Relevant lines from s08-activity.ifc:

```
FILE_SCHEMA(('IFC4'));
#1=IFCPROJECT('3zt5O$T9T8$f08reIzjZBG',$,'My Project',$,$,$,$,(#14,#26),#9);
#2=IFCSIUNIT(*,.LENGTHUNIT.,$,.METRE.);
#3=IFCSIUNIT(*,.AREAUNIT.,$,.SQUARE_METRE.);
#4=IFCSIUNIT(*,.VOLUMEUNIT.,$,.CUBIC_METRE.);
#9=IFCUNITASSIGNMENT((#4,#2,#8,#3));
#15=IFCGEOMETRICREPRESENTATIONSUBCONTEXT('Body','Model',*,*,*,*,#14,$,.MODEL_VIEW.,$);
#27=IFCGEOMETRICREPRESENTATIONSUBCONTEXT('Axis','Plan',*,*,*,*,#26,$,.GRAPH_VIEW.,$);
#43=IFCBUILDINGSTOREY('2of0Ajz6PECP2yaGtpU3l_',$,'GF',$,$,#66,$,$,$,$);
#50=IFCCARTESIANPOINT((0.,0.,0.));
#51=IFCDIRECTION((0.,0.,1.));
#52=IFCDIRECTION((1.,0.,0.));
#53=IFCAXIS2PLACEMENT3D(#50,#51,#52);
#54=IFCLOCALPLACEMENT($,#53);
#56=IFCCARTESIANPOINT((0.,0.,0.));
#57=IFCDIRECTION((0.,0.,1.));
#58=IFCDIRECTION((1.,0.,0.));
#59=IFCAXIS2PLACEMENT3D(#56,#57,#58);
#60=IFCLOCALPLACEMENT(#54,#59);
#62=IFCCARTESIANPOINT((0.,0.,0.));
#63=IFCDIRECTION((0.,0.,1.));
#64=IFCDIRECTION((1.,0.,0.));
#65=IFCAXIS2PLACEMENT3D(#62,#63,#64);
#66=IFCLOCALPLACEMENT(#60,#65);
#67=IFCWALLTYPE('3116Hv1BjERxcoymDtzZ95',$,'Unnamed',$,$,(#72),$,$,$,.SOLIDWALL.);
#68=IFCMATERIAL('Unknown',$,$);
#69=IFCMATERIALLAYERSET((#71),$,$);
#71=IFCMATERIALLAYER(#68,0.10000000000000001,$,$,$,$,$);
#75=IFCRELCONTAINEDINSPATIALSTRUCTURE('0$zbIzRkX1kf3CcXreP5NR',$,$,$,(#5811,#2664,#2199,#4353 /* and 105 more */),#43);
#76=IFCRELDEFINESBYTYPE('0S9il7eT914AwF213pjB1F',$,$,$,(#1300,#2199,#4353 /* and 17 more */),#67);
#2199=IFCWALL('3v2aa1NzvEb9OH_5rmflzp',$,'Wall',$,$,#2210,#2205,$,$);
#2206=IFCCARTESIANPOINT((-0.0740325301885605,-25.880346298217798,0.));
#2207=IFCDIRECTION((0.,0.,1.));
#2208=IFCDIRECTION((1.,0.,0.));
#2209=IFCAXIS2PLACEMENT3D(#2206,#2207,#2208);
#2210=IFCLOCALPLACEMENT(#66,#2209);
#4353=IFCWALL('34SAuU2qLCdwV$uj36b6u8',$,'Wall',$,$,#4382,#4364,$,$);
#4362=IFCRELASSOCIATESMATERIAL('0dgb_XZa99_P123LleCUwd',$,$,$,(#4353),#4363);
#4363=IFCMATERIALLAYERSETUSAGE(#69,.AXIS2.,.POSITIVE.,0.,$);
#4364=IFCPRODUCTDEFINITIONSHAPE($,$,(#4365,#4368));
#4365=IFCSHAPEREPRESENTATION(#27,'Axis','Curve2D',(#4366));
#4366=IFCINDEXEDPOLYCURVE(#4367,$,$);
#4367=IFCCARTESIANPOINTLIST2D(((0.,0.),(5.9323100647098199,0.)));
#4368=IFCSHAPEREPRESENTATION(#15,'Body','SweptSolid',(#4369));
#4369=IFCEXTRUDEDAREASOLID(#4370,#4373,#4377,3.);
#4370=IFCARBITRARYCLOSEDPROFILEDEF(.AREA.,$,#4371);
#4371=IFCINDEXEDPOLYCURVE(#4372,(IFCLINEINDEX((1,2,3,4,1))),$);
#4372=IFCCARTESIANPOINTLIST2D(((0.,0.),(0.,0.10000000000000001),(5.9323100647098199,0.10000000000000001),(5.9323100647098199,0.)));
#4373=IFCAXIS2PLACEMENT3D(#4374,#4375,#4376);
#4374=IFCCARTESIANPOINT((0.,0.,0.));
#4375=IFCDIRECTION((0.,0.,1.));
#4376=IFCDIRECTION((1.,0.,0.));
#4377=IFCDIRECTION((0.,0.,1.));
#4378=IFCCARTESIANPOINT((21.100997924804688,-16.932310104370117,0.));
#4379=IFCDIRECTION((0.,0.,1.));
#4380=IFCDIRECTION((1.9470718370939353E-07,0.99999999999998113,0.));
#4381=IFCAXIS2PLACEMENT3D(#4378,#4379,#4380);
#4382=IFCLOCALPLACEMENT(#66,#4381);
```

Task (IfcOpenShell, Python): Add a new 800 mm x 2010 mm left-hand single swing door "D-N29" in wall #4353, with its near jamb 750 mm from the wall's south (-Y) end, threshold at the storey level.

```python
import numpy as np
import ifcopenshell
import ifcopenshell.api.feature
import ifcopenshell.api.geometry
import ifcopenshell.api.root
import ifcopenshell.api.spatial
import ifcopenshell.geom
import ifcopenshell.util.element
import ifcopenshell.util.placement
import ifcopenshell.util.representation
import ifcopenshell.util.shape
import ifcopenshell.util.unit

model = ifcopenshell.open("s08-activity.ifc")
unit_scale = ifcopenshell.util.unit.calculate_unit_scale(model)
settings = ifcopenshell.geom.settings()


def volume(element):
    """Net volume in cubic metres, openings subtracted."""
    shape = ifcopenshell.geom.create_shape(settings, element)
    return ifcopenshell.util.shape.get_volume(shape.geometry)


wall = model.by_id(4353)
storey = ifcopenshell.util.element.get_container(wall, ifc_class="IfcBuildingStorey")
context = ifcopenshell.util.representation.get_context(model, "Model", "Body", "MODEL_VIEW")
before = volume(wall)

width, height, from_end, sill = 0.8, 2.01, 0.75, 0.0  # metres

# The wall runs along its own X axis, and the end named is its -X end.
wall_shape = ifcopenshell.geom.create_shape(settings, wall)
x, y, z = ifcopenshell.util.shape.get_vertices(wall_shape.geometry).T
start = x.min() + from_end
face, thickness = float(y.min()), float(y.max() - y.min())
wall_matrix = ifcopenshell.util.placement.get_local_placement(wall.ObjectPlacement)
level = ifcopenshell.util.placement.get_local_placement(storey.ObjectPlacement)[2, 3]


def in_wall(x, y):
    """Placement at x, y metres in the wall's axes, at sill height."""
    matrix = wall_matrix.copy()
    matrix[:, 3] = wall_matrix @ np.array([x / unit_scale, y / unit_scale, 0.0, 1.0])
    matrix[2, 3] = level + sill / unit_scale
    return matrix


# Opening: a box that overshoots both wall faces by 50 mm.
opening = ifcopenshell.api.root.create_entity(model, ifc_class="IfcOpeningElement", predefined_type="OPENING")
box = ifcopenshell.api.geometry.add_wall_representation(
    model, context=context, length=width, height=height, thickness=thickness + 0.1
)
ifcopenshell.api.geometry.assign_representation(model, product=opening, representation=box)
ifcopenshell.api.geometry.edit_object_placement(model, product=opening, matrix=in_wall(start, face - 0.05), is_si=False)
ifcopenshell.api.feature.add_feature(model, feature=opening, element=wall)

door = ifcopenshell.api.root.create_entity(model, ifc_class="IfcDoor", name="D-N29", predefined_type="DOOR")
door.OverallWidth, door.OverallHeight = width / unit_scale, height / unit_scale
door.OperationType = "SINGLE_SWING_LEFT"
body = ifcopenshell.api.geometry.add_door_representation(
    model,
    context=context,
    overall_width=door.OverallWidth,
    overall_height=door.OverallHeight,
    operation_type="SINGLE_SWING_LEFT",
    lining_properties={"LiningDepth": thickness / unit_scale, "ThresholdDepth": thickness / unit_scale},
)
ifcopenshell.api.geometry.assign_representation(model, product=door, representation=body)
ifcopenshell.api.spatial.assign_container(model, products=[door], relating_structure=storey)
ifcopenshell.api.feature.add_filling(model, opening=opening, element=door)

# The lining spans the wall, so the door starts at the wall face.
ifcopenshell.api.geometry.edit_object_placement(model, product=door, matrix=in_wall(start, face), is_si=False)

after = volume(wall)

print(f"wall volume {before:.3f} -> {after:.3f} m3")

model.write("s08-activity_rev.ifc")
```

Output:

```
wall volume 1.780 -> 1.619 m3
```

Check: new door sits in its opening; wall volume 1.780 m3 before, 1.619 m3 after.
